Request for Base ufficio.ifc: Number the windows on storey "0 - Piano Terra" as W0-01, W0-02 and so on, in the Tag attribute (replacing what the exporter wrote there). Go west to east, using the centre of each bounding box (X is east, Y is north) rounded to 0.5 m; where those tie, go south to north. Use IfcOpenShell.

First a look at what the model holds.

```python
import ifcopenshell
import ifcopenshell.util.element
import ifcopenshell.util.placement

model = ifcopenshell.open("Base ufficio.ifc")
print(model.schema)
storey = next(s for s in model.by_type("IfcBuildingStorey") if s.Name == "0 - Piano Terra")
windows = [e for e in ifcopenshell.util.element.get_decomposition(storey) if e.is_a("IfcWindow")]
for e in sorted(windows, key=lambda e: e.id()):
    origin = ifcopenshell.util.placement.get_local_placement(e.ObjectPlacement)[:3, 3]
    print(e.id(), e.Tag, e.Name, origin.round(2) + 0.0, sep=" | ")
```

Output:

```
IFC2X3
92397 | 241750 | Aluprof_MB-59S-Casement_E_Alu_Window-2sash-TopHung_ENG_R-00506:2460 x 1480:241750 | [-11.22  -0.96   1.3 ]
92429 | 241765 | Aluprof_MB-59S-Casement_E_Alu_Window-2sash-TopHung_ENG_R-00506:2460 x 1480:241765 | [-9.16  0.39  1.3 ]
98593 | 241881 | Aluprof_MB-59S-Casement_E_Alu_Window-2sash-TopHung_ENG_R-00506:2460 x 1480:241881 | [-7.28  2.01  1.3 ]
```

```python
import ifcopenshell
import ifcopenshell.geom
import ifcopenshell.util.element
import ifcopenshell.util.shape

model = ifcopenshell.open("Base ufficio.ifc")
settings = ifcopenshell.geom.settings()
settings.set("use-world-coords", True)


def centre(element):
    shape = ifcopenshell.geom.create_shape(settings, element)
    return ifcopenshell.util.shape.get_bbox_centroid(shape.geometry)


storey = next(s for s in model.by_type("IfcBuildingStorey") if s.Name == "0 - Piano Terra")
windows = [e for e in ifcopenshell.util.element.get_decomposition(storey) if e.is_a("IfcWindow")]

# Insertion points can sit at a corner or the storey origin, so sort by the geometry (in metres).
centres = {e: centre(e) for e in windows}
windows.sort(key=lambda e: (round(centres[e][0] / 0.5), centres[e][1]))

for i, e in enumerate(windows, start=1):
    number = f"W0-{i:02d}"
    e.Tag = number
    print(e.id(), number)

model.write("Base ufficio-out.ifc")
```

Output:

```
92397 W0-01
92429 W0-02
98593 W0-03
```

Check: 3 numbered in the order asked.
